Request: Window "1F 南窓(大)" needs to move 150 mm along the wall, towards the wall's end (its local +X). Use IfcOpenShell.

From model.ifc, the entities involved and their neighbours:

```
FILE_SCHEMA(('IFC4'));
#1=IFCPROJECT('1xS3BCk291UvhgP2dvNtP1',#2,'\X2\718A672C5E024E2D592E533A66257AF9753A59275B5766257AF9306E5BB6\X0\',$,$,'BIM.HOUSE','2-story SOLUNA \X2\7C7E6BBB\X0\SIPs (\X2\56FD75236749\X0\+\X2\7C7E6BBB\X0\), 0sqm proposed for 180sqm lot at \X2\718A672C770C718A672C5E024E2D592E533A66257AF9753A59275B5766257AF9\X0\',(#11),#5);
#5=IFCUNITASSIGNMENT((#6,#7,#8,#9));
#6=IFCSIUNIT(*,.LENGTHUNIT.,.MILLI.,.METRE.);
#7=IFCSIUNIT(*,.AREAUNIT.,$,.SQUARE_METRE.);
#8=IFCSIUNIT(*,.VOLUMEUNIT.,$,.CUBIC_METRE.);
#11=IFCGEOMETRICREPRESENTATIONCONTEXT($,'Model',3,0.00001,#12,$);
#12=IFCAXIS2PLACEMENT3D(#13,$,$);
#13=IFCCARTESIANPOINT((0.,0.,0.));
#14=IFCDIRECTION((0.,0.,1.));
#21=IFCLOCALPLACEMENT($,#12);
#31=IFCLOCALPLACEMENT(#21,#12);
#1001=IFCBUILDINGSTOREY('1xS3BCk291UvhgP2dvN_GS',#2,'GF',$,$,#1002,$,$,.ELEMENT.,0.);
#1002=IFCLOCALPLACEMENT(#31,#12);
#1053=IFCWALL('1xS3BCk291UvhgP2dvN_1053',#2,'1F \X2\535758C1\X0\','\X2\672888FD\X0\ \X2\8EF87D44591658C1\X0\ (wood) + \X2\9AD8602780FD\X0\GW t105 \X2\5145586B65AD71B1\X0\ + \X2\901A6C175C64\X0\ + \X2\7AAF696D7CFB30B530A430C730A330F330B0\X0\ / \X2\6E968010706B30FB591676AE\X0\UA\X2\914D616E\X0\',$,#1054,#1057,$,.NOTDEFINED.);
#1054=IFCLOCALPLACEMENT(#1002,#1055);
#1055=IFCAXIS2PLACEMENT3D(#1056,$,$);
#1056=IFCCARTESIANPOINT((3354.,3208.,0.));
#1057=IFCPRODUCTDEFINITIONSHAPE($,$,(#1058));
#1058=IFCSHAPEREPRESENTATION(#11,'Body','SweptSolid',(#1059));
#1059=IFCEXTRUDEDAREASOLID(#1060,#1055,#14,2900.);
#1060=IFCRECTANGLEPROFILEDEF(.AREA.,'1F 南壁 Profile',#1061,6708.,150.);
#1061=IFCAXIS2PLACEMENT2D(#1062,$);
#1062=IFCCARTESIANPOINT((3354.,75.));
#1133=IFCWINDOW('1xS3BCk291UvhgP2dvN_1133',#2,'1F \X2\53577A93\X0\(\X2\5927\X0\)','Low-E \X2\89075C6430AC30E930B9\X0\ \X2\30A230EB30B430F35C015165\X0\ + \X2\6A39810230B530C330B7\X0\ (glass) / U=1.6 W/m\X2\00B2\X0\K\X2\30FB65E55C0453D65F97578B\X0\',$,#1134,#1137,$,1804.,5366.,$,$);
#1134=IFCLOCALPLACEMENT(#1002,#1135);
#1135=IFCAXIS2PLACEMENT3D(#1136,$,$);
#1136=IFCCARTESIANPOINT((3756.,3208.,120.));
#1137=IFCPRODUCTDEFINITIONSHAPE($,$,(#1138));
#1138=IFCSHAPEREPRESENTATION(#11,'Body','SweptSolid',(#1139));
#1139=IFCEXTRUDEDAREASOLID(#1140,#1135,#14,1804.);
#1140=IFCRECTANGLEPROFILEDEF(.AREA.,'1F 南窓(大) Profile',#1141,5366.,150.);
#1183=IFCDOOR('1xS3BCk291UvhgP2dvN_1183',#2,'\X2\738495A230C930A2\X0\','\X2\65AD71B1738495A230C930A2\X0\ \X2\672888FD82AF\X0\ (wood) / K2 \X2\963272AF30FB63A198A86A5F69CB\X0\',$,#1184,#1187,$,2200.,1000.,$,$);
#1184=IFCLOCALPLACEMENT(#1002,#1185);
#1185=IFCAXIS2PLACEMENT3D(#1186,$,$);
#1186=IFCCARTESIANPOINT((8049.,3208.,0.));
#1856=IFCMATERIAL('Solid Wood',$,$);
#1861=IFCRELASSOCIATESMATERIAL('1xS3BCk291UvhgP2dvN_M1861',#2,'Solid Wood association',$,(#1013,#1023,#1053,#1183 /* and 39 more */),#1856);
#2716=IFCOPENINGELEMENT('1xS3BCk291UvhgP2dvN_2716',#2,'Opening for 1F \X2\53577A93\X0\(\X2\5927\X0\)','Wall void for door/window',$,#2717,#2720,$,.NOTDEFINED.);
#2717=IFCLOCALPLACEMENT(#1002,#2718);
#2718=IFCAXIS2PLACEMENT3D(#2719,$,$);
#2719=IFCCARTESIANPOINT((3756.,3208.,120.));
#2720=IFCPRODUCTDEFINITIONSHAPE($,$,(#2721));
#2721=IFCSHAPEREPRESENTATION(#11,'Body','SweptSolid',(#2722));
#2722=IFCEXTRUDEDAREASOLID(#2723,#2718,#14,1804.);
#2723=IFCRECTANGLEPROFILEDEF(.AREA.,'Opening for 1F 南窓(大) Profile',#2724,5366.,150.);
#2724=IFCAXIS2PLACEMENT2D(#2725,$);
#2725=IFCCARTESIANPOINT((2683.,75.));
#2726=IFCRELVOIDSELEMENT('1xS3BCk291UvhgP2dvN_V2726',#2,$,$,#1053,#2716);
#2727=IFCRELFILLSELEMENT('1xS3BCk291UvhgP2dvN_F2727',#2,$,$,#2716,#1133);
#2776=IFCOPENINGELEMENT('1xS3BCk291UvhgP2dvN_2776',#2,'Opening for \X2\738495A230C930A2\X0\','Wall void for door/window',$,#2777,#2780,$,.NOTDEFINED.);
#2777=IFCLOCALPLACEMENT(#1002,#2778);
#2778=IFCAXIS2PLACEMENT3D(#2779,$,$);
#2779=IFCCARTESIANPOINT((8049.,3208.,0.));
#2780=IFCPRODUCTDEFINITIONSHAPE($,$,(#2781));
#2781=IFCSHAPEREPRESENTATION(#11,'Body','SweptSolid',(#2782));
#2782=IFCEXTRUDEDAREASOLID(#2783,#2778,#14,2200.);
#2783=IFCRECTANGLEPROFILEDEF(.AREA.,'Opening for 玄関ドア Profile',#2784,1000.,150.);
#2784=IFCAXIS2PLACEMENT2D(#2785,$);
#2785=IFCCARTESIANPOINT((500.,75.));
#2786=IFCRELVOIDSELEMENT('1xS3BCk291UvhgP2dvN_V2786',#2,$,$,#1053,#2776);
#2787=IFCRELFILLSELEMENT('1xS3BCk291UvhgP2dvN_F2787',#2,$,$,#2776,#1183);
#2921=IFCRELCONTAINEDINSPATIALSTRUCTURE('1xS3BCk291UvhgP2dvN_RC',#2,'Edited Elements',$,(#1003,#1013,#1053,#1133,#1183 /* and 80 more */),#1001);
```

```python
import ifcopenshell
import ifcopenshell.api.geometry
import ifcopenshell.util.placement
import ifcopenshell.util.unit

model = ifcopenshell.open("model.ifc")
unit_scale = ifcopenshell.util.unit.calculate_unit_scale(model)

window = model.by_guid("1xS3BCk291UvhgP2dvN_1133")
opening = window.FillsVoids[0].RelatingOpeningElement
wall = opening.VoidsElements[0].RelatingBuildingElement

wall_matrix = ifcopenshell.util.placement.get_local_placement(wall.ObjectPlacement)
shift = wall_matrix[:3, 0] * 0.15 / unit_scale
before = ifcopenshell.util.placement.get_local_placement(window.ObjectPlacement)[:3, 3].copy()

# The window is not placed relative to its opening, so move both.
for product in (opening, window):
    matrix = ifcopenshell.util.placement.get_local_placement(product.ObjectPlacement)
    matrix[:3, 3] += shift
    ifcopenshell.api.geometry.edit_object_placement(model, product=product, matrix=matrix, is_si=False)

after = ifcopenshell.util.placement.get_local_placement(window.ObjectPlacement)[:3, 3]
print("window moved by", (after - before).round(3) + 0.0)

model.write("model_v2.ifc")
```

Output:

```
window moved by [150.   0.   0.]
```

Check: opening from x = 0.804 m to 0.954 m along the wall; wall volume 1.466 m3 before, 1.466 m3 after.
